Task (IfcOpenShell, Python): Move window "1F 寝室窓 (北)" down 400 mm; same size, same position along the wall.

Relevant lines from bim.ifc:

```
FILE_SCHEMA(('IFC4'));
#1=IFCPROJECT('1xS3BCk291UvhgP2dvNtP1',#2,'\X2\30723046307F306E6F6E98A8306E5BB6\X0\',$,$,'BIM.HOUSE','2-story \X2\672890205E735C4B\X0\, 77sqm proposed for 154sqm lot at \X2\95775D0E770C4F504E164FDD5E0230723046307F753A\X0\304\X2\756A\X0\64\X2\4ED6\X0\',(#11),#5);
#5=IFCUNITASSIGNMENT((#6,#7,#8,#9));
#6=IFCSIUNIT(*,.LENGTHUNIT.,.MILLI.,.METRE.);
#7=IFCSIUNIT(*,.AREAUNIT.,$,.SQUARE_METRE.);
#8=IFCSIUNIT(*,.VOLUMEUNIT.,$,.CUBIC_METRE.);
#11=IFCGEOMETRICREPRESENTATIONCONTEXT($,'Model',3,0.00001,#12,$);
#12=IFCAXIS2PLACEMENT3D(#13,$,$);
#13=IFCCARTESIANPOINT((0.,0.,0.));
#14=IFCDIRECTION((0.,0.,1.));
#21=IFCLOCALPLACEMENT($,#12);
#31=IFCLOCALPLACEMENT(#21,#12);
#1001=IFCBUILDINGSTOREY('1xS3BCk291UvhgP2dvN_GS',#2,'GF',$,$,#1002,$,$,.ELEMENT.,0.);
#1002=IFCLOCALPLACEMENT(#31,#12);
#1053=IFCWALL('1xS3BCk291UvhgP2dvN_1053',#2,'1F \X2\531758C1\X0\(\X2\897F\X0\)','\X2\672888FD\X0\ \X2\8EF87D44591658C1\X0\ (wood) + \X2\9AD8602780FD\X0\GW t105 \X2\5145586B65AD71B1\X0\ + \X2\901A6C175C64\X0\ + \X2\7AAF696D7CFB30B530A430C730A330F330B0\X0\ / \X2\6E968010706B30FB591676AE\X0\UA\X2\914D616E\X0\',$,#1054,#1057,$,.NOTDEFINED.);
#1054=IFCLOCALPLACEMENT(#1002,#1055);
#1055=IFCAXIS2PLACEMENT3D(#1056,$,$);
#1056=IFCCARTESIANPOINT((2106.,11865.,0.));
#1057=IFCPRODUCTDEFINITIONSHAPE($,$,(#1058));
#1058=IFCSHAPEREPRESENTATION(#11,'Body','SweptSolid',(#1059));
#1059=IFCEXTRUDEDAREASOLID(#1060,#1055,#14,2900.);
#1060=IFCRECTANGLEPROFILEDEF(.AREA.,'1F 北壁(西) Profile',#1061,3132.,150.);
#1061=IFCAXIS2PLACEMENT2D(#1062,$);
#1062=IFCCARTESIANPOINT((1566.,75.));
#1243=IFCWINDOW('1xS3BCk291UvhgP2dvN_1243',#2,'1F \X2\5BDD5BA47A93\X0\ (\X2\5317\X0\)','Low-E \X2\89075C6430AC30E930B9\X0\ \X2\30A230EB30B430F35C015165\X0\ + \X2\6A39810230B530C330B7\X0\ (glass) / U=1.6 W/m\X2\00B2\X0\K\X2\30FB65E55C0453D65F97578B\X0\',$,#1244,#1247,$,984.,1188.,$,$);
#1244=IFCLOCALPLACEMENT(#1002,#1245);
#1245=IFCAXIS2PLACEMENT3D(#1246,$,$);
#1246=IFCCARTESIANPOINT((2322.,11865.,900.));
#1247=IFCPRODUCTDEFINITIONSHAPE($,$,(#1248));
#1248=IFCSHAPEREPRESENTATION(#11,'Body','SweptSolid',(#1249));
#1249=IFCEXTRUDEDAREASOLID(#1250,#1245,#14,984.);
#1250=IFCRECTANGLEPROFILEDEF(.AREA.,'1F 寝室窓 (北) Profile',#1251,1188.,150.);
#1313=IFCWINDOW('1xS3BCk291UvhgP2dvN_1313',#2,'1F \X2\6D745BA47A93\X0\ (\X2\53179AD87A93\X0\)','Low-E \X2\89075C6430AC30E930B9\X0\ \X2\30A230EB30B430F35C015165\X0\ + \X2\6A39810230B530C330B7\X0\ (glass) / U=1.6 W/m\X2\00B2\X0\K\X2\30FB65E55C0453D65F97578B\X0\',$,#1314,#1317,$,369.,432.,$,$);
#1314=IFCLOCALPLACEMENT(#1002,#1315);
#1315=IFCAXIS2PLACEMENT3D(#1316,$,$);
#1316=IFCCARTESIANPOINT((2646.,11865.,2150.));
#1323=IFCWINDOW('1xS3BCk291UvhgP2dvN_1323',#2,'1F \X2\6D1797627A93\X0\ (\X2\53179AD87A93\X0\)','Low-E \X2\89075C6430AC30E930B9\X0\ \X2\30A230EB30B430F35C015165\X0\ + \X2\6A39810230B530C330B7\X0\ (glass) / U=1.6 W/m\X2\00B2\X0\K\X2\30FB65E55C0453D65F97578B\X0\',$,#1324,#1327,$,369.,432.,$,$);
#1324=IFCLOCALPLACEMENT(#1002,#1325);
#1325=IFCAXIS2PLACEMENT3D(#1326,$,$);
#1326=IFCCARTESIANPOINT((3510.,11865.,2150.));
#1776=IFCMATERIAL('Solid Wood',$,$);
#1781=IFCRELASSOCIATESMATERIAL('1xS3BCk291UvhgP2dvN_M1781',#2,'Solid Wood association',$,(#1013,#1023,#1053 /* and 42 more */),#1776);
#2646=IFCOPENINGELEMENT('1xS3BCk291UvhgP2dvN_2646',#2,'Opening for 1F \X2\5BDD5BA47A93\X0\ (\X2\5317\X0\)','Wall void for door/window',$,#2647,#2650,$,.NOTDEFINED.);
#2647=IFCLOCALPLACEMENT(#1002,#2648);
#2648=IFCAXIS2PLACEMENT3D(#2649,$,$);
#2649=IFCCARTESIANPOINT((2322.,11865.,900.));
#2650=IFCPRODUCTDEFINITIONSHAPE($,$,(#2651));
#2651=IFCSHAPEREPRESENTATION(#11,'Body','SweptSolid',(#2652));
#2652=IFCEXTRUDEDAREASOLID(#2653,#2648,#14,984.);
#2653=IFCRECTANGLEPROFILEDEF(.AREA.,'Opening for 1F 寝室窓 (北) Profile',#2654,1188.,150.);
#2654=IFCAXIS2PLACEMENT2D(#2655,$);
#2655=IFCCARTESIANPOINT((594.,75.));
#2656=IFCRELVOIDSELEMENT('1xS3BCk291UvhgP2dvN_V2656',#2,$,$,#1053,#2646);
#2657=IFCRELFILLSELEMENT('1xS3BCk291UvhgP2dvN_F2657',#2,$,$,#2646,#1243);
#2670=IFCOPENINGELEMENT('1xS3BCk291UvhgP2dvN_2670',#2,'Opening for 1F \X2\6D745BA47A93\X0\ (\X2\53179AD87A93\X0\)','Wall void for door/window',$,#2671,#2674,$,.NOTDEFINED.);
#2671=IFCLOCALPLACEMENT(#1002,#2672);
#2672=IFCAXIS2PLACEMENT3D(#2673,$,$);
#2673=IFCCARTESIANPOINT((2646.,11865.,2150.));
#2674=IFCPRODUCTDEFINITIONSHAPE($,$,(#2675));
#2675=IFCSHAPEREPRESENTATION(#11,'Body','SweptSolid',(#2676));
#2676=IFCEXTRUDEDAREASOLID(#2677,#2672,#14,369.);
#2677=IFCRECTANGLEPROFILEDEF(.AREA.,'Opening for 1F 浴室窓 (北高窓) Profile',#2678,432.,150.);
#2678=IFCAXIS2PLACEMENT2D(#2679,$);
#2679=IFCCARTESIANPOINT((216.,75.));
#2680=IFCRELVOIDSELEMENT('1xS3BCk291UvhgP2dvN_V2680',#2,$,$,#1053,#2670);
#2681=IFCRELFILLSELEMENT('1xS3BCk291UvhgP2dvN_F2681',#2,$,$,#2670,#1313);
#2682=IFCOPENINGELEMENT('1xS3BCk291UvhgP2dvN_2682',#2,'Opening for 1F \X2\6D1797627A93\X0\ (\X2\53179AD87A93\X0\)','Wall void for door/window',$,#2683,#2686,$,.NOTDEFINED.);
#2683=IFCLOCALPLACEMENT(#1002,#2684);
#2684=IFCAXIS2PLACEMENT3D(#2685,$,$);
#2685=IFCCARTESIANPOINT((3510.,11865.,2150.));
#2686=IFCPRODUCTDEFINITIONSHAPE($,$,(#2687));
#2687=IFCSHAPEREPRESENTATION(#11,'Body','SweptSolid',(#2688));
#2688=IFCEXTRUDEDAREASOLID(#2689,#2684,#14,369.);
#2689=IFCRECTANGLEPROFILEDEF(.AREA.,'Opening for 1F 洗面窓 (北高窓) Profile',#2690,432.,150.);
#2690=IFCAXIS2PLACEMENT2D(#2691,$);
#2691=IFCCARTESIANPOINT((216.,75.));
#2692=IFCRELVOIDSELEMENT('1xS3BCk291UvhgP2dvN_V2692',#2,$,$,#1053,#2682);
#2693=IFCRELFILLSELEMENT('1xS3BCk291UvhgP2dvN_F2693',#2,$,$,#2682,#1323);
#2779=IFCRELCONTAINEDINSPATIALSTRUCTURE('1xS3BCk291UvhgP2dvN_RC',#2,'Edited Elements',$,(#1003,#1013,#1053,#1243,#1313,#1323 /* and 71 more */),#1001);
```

```python
import numpy as np
import ifcopenshell
import ifcopenshell.api.geometry
import ifcopenshell.util.placement
import ifcopenshell.util.unit

model = ifcopenshell.open("bim.ifc")
unit_scale = ifcopenshell.util.unit.calculate_unit_scale(model)

window = model.by_guid("1xS3BCk291UvhgP2dvN_1243")
opening = window.FillsVoids[0].RelatingOpeningElement
dz = -0.4 / unit_scale

shift = np.array([0.0, 0.0, dz])
# The window is not placed relative to its opening, so move both.
for product in (opening, window):
    matrix = ifcopenshell.util.placement.get_local_placement(product.ObjectPlacement)
    matrix[:3, 3] += shift
    ifcopenshell.api.geometry.edit_object_placement(model, product=product, matrix=matrix, is_si=False)

print(f"moved by {dz * unit_scale:+.3f} m")

model.write("bim_updated.ifc")
```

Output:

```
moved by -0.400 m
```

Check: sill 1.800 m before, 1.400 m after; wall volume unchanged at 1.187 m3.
